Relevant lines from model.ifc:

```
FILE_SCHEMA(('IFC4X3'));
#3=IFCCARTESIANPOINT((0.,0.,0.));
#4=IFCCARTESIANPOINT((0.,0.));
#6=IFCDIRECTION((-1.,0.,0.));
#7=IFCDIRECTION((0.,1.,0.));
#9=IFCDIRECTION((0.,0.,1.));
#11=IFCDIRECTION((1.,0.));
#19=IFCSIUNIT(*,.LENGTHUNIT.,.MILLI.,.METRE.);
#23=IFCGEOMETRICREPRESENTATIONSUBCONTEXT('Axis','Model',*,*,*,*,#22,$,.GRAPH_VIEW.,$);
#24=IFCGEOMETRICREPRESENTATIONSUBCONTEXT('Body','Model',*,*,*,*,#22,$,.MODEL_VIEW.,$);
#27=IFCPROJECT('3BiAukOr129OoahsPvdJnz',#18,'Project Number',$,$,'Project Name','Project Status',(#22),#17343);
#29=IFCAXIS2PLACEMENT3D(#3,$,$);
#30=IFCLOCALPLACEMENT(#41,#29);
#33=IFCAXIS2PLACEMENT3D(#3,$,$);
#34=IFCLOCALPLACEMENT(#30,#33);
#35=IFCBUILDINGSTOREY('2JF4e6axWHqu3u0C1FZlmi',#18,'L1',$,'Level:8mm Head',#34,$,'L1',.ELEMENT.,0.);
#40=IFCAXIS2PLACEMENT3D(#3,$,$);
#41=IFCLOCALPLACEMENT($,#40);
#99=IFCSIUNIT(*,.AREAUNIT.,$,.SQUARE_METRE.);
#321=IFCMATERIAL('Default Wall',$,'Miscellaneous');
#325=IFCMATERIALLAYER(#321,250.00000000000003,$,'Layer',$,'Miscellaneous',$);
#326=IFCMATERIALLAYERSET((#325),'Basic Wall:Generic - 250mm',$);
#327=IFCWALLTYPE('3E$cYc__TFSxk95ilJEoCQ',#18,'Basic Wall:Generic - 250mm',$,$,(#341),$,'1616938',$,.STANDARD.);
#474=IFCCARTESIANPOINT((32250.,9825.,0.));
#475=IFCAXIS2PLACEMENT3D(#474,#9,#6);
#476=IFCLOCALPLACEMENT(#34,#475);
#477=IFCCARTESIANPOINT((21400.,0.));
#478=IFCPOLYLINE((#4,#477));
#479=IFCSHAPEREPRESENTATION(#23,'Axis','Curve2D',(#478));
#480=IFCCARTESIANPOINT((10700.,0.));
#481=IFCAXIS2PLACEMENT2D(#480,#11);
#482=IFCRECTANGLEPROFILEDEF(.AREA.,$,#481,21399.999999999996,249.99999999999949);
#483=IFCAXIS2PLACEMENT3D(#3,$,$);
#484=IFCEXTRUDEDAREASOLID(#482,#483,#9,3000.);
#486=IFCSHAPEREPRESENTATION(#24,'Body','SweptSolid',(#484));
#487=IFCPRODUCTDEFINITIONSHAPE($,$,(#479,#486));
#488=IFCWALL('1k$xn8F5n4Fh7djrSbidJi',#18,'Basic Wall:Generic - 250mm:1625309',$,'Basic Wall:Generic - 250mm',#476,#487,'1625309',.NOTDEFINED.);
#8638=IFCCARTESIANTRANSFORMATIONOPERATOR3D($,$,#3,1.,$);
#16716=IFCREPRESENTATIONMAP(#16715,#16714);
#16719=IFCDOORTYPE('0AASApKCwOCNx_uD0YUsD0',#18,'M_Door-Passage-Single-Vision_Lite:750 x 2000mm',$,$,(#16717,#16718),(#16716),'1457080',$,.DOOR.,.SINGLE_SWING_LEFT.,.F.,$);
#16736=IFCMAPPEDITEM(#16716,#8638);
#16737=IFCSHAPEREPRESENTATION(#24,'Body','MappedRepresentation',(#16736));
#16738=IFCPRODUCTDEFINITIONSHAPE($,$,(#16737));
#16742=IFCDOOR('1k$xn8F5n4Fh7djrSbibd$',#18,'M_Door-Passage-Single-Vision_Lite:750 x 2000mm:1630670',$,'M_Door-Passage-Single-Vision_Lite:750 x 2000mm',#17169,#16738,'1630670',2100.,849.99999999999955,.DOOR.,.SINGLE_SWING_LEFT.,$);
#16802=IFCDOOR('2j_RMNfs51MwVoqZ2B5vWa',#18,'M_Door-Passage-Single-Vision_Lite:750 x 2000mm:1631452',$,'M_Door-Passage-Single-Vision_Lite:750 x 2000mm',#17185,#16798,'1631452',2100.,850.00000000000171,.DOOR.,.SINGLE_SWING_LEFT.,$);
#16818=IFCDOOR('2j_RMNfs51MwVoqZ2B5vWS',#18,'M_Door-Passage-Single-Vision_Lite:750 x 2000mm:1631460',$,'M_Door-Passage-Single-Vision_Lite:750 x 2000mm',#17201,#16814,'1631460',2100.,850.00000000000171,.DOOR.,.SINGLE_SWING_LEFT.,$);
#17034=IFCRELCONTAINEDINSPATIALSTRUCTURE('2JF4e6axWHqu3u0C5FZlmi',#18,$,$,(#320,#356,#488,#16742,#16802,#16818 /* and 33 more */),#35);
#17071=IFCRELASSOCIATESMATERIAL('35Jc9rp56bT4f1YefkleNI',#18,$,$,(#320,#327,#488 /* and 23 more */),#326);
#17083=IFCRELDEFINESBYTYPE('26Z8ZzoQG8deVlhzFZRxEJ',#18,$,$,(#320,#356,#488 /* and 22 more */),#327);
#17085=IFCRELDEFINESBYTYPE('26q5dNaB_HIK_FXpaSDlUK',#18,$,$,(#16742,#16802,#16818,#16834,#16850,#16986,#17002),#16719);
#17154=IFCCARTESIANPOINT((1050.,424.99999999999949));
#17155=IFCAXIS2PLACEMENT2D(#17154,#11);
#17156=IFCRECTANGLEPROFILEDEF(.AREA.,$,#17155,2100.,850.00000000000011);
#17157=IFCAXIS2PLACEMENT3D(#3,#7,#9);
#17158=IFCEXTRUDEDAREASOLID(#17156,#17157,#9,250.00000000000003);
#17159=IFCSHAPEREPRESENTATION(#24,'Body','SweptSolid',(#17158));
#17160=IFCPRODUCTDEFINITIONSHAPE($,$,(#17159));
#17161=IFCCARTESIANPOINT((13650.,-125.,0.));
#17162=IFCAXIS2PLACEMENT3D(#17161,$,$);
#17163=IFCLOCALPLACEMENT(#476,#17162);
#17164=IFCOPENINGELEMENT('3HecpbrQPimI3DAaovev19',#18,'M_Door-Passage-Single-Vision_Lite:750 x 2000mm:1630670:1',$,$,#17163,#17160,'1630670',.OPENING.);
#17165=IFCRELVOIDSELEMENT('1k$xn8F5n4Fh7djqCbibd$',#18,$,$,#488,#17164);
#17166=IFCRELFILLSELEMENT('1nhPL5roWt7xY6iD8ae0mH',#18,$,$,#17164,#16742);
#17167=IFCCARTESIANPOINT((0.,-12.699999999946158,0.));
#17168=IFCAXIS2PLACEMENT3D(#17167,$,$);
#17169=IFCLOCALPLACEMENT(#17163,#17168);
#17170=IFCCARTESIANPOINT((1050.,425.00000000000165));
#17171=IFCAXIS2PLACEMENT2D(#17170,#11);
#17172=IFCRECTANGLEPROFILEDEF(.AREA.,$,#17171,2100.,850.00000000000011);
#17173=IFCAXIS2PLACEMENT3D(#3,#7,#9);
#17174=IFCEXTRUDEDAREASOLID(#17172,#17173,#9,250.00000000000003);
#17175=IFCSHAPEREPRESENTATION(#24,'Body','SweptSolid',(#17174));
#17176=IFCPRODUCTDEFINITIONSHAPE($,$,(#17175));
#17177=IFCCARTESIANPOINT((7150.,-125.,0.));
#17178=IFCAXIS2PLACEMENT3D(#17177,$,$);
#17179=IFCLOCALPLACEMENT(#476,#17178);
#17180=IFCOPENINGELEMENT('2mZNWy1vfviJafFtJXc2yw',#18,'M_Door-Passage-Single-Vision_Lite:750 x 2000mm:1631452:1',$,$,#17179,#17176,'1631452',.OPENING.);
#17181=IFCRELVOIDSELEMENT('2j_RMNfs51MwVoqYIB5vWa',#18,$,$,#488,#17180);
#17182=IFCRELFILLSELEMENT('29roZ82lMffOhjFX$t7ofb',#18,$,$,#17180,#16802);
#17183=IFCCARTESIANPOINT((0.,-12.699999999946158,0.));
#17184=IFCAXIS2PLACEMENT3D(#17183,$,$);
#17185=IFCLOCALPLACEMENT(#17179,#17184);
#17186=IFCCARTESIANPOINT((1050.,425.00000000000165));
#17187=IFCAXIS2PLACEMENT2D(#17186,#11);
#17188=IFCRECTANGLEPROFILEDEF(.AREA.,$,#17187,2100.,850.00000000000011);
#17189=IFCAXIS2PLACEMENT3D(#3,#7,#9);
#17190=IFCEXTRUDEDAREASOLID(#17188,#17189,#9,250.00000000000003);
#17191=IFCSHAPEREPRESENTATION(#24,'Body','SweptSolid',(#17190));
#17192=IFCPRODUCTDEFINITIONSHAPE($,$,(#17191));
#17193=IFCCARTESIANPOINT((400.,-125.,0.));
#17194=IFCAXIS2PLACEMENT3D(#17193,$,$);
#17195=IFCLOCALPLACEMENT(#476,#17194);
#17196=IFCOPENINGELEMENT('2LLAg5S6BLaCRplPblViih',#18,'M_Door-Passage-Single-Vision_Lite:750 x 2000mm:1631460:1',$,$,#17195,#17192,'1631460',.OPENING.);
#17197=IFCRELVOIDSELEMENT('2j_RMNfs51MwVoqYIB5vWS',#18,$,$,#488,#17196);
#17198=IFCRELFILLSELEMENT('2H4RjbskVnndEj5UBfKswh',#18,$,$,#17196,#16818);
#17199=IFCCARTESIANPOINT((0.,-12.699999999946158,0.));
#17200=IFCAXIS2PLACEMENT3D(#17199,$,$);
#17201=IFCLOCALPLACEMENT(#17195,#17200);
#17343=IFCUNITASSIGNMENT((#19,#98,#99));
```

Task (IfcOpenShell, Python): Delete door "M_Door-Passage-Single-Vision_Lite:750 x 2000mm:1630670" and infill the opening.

```python
import ifcopenshell
import ifcopenshell.api.feature
import ifcopenshell.api.root
import ifcopenshell.geom
import ifcopenshell.util.shape

model = ifcopenshell.open("model.ifc")
settings = ifcopenshell.geom.settings()


def volume(element):
    """Net volume in cubic metres, openings subtracted."""
    shape = ifcopenshell.geom.create_shape(settings, element)
    return ifcopenshell.util.shape.get_volume(shape.geometry)


door = model.by_guid("1k$xn8F5n4Fh7djrSbibd$")
opening = door.FillsVoids[0].RelatingOpeningElement
wall = opening.VoidsElements[0].RelatingBuildingElement
before = volume(wall)

ifcopenshell.api.root.remove_product(model, product=door)
ifcopenshell.api.feature.remove_feature(model, feature=opening)

after = volume(wall)

print(f"wall volume {before:.3f} -> {after:.3f} m3")

model.write("model_rev.ifc")
```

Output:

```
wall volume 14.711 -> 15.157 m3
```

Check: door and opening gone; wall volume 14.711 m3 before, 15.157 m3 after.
